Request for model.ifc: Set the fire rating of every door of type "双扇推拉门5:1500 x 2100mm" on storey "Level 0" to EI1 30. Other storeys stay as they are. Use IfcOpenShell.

First a look at what the model holds.

```python
import ifcopenshell
import ifcopenshell.util.element

model = ifcopenshell.open("model.ifc")
print(model.schema)
storey = next(s for s in model.by_type("IfcBuildingStorey") if s.Name == "Level 0")
doors = [e for e in ifcopenshell.util.element.get_decomposition(storey) if e.is_a("IfcDoor")]
seen = {}
for e in doors:
    element_type = ifcopenshell.util.element.get_type(e)
    key = (element_type.Name if element_type != e and element_type else None, ifcopenshell.util.element.get_pset(e, "Pset_DoorCommon", "FireRating"))
    seen[key] = seen.get(key, 0) + 1
for (name, value), count in sorted(seen.items(), key=str):
    print(count, "x", name, "|", value)
```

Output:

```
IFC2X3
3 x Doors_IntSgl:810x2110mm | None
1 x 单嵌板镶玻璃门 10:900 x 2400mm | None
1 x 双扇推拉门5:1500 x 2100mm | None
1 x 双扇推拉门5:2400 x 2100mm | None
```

```python
import ifcopenshell
import ifcopenshell.api.pset
import ifcopenshell.util.element

model = ifcopenshell.open("model.ifc")

storey = next(s for s in model.by_type("IfcBuildingStorey") if s.Name == "Level 0")
doors = [e for e in ifcopenshell.util.element.get_decomposition(storey) if e.is_a("IfcDoor")]

count = 0
for e in doors:
    element_type = ifcopenshell.util.element.get_type(e)
    if element_type in (None, e) or element_type.Name != "双扇推拉门5:1500 x 2100mm":
        continue
    # add_pset returns the element's existing set when there is one.
    pset = ifcopenshell.api.pset.add_pset(model, product=e, name="Pset_DoorCommon")
    ifcopenshell.api.pset.edit_pset(model, pset=pset, properties={"FireRating": "EI1 30"})
    count += 1

print(count, "doors updated")

model.write("model-out.ifc")
```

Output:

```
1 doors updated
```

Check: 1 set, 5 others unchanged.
